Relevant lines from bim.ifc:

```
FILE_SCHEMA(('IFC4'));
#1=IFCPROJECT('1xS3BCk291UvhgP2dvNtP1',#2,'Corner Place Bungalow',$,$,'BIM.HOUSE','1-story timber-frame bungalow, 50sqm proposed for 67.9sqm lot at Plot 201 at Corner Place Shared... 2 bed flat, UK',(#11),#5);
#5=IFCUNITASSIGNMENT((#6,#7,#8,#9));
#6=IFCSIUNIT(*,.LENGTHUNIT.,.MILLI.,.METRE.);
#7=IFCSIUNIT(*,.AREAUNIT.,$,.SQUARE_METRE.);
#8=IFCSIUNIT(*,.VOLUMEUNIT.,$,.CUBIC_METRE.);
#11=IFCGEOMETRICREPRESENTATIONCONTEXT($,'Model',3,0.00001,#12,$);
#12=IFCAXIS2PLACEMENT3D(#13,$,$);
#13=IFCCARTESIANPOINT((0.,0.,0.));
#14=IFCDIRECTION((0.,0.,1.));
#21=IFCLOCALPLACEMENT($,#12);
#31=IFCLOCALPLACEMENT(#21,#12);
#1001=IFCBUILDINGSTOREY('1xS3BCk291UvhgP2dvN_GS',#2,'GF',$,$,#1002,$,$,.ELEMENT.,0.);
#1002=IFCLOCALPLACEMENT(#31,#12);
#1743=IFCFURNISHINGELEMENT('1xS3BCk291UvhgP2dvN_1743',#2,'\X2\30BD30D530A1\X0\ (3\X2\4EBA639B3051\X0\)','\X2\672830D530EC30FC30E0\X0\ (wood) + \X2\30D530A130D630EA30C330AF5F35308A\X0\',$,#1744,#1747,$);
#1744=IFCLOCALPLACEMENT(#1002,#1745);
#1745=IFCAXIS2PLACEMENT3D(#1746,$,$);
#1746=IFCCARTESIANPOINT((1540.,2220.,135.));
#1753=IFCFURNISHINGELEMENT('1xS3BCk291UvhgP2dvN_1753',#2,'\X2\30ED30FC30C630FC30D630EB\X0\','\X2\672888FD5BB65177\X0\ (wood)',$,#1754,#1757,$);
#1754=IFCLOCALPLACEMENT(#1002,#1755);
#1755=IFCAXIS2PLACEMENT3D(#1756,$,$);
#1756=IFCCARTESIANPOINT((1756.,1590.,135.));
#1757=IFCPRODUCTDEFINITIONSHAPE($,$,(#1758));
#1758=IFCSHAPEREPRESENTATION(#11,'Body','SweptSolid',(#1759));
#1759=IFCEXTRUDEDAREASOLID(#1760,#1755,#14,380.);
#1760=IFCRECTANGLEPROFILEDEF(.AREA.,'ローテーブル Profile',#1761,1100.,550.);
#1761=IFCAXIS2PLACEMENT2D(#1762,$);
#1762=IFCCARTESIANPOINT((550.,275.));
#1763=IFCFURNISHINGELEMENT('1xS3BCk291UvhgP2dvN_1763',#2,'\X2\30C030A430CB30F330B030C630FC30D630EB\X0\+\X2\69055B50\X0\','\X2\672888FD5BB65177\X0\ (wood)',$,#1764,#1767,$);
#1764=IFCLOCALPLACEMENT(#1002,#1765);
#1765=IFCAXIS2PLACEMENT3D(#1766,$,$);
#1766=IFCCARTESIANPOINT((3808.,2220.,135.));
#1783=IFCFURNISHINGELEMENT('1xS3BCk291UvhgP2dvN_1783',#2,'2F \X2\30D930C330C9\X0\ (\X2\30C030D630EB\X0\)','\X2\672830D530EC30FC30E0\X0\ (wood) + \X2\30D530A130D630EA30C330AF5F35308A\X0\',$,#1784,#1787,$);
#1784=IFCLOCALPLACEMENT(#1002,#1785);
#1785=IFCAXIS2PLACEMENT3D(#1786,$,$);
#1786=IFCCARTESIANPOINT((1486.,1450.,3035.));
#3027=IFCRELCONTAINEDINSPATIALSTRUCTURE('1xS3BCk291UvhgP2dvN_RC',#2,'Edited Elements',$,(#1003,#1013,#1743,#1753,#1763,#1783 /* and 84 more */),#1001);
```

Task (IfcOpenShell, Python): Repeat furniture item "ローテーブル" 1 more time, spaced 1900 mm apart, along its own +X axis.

```python
import ifcopenshell
import ifcopenshell.api.geometry
import ifcopenshell.api.root
import ifcopenshell.util.element
import ifcopenshell.util.placement

model = ifcopenshell.open("bim.ifc")


def reuse_history(source, copy):
    """copy_class also copies each property set's owner history, people and application; keep the originals."""
    for rel in copy.IsDefinedBy:
        if rel.is_a("IfcRelDefinesByProperties") and (history := rel.RelatingPropertyDefinition.OwnerHistory):
            rel.RelatingPropertyDefinition.OwnerHistory = source.OwnerHistory
            ifcopenshell.util.element.remove_deep2(model, history)


source = model.by_guid("1xS3BCk291UvhgP2dvN_1753")
base = ifcopenshell.util.placement.get_local_placement(source.ObjectPlacement)
step = base[:3, 0] * 1900.0

for i in range(1, 2):
    copy = ifcopenshell.api.root.copy_class(model, product=source)
    copy.Representation = ifcopenshell.util.element.copy_deep(
        model, source.Representation, exclude=["IfcGeometricRepresentationContext", "IfcRepresentationMap"]
    )
    reuse_history(source, copy)
    matrix = base.copy()
    matrix[:3, 3] += i * step
    print("added at", matrix[:3, 3].round(3) + 0.0)
    ifcopenshell.api.geometry.edit_object_placement(model, product=copy, matrix=matrix, is_si=False)

model.write("bim_rev.ifc")
```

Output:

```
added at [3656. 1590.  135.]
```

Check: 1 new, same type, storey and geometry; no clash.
